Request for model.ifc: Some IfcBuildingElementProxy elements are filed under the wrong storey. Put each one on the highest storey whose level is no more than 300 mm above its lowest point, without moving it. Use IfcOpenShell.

First a look at what the model holds.

```python
import ifcopenshell
import ifcopenshell.util.element
import ifcopenshell.util.placement

model = ifcopenshell.open("model.ifc")
print(model.schema)
for storey in model.by_type("IfcBuildingStorey"):
    level = ifcopenshell.util.placement.get_storey_elevation(storey)
    count = sum(e.is_a("IfcBuildingElementProxy") for e in ifcopenshell.util.element.get_contained(storey))
    print(storey.id(), storey.Name, round(level, 3), count, sep=" | ")
```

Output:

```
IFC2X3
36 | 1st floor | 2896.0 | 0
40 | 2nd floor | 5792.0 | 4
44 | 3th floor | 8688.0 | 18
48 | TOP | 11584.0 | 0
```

```python
import ifcopenshell
import ifcopenshell.api.spatial
import ifcopenshell.geom
import ifcopenshell.util.element
import ifcopenshell.util.placement
import ifcopenshell.util.shape
import ifcopenshell.util.unit

model = ifcopenshell.open("model.ifc")
unit_scale = ifcopenshell.util.unit.calculate_unit_scale(model)
settings = ifcopenshell.geom.settings()

levels = sorted(
    ((ifcopenshell.util.placement.get_storey_elevation(s) * unit_scale, s) for s in model.by_type("IfcBuildingStorey")),
    key=lambda pair: pair[0],
)

for e in model.by_type("IfcBuildingElementProxy"):
    current = e.ContainedInStructure[0].RelatingStructure if e.ContainedInStructure else None
    if current is None or not current.is_a("IfcBuildingStorey"):
        continue
    shape = ifcopenshell.geom.create_shape(settings, e)
    bottom = ifcopenshell.util.shape.get_shape_bottom_elevation(shape, shape.geometry)
    below = [s for level, s in levels if level <= bottom + 0.3]
    storey = below[-1] if below else levels[0][1]
    if storey != current:
        # assign_container keeps the world position.
        ifcopenshell.api.spatial.assign_container(model, products=[e], relating_structure=storey)
        print(e.id(), current.Name, "->", storey.Name)

model.write("model_rev.ifc")
```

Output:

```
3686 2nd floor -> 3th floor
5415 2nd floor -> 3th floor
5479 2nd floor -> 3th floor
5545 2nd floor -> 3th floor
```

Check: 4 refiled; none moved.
